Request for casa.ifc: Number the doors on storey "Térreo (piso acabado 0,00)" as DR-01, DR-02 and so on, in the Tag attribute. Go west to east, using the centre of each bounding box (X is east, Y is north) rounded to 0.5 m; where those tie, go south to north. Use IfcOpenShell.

First a look at what the model holds.

```python
import ifcopenshell
import ifcopenshell.util.element
import ifcopenshell.util.placement

model = ifcopenshell.open("casa.ifc")
print(model.schema)
storey = next(s for s in model.by_type("IfcBuildingStorey") if s.Name == "Térreo (piso acabado 0,00)")
doors = [e for e in ifcopenshell.util.element.get_decomposition(storey) if e.is_a("IfcDoor")]
for e in sorted(doors, key=lambda e: e.id()):
    origin = ifcopenshell.util.placement.get_local_placement(e.ObjectPlacement)[:3, 3]
    print(e.id(), e.Tag, e.Name, origin.round(2) + 0.0, sep=" | ")
```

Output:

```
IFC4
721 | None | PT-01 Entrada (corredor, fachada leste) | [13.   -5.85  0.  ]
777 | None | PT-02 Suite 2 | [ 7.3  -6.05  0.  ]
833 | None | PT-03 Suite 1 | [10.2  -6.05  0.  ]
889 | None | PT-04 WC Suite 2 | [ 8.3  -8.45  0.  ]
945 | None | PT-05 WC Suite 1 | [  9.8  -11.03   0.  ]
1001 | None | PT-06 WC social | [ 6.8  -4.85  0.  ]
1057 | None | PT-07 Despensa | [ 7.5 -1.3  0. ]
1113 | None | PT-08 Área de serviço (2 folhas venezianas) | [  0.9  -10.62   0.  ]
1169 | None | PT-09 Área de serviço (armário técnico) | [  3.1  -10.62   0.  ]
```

```python
import ifcopenshell
import ifcopenshell.geom
import ifcopenshell.util.element
import ifcopenshell.util.shape

model = ifcopenshell.open("casa.ifc")
settings = ifcopenshell.geom.settings()
settings.set("use-world-coords", True)


def centre(element):
    shape = ifcopenshell.geom.create_shape(settings, element)
    return ifcopenshell.util.shape.get_bbox_centroid(shape.geometry)


storey = next(s for s in model.by_type("IfcBuildingStorey") if s.Name == "Térreo (piso acabado 0,00)")
doors = [e for e in ifcopenshell.util.element.get_decomposition(storey) if e.is_a("IfcDoor")]

# Insertion points can sit at a corner or the storey origin, so sort by the geometry (in metres).
centres = {e: centre(e) for e in doors}
doors.sort(key=lambda e: (round(centres[e][0] / 0.5), centres[e][1]))

for i, e in enumerate(doors, start=1):
    number = f"DR-{i:02d}"
    e.Tag = number
    print(e.id(), number)

model.write("casa_updated.ifc")
```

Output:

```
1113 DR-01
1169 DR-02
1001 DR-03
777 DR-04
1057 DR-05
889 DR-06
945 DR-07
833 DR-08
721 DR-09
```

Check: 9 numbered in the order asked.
